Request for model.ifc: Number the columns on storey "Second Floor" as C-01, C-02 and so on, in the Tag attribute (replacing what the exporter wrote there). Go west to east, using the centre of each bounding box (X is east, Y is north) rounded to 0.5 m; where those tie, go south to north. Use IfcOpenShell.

First a look at what the model holds.

```python
import ifcopenshell
import ifcopenshell.util.element
import ifcopenshell.util.placement

model = ifcopenshell.open("model.ifc")
print(model.schema)
storey = next(s for s in model.by_type("IfcBuildingStorey") if s.Name == "Second Floor")
columns = [e for e in ifcopenshell.util.element.get_decomposition(storey) if e.is_a("IfcColumn")]
for e in sorted(columns, key=lambda e: e.id()):
    origin = ifcopenshell.util.placement.get_local_placement(e.ObjectPlacement)[:3, 3]
    print(e.id(), e.Tag, e.Name, origin.round(2) + 0.0, sep=" | ")
```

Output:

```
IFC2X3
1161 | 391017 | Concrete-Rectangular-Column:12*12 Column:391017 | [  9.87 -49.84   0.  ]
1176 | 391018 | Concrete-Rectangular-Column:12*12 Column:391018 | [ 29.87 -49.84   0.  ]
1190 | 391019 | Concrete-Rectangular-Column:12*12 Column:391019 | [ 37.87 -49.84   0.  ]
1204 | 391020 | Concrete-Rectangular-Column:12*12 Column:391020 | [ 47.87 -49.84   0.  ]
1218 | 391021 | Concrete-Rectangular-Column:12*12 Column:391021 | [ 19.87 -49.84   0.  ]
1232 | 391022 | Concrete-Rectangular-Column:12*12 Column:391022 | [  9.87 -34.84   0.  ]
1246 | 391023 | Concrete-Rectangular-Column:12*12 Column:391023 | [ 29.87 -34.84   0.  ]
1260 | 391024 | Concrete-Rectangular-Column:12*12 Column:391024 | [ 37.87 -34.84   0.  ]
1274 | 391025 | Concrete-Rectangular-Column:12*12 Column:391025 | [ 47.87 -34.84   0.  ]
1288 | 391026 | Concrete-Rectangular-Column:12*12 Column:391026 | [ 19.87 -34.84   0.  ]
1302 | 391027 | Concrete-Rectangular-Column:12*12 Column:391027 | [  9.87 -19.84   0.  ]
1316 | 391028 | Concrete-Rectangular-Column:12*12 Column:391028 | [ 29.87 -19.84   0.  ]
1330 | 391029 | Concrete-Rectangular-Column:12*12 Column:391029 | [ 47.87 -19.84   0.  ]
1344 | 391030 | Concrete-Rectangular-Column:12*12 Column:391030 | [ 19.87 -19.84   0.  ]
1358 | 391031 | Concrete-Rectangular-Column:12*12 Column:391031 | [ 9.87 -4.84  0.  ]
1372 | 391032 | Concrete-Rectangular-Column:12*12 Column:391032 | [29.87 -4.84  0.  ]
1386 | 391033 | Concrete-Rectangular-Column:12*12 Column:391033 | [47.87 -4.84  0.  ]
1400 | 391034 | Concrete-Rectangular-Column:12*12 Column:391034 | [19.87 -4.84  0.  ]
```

```python
import ifcopenshell
import ifcopenshell.geom
import ifcopenshell.util.element
import ifcopenshell.util.shape

model = ifcopenshell.open("model.ifc")
settings = ifcopenshell.geom.settings()
settings.set("use-world-coords", True)


def centre(element):
    shape = ifcopenshell.geom.create_shape(settings, element)
    return ifcopenshell.util.shape.get_bbox_centroid(shape.geometry)


storey = next(s for s in model.by_type("IfcBuildingStorey") if s.Name == "Second Floor")
columns = [e for e in ifcopenshell.util.element.get_decomposition(storey) if e.is_a("IfcColumn")]

# Insertion points can sit at a corner or the storey origin, so sort by the geometry (in metres).
centres = {e: centre(e) for e in columns}
columns.sort(key=lambda e: (round(centres[e][0] / 0.5), centres[e][1]))

for i, e in enumerate(columns, start=1):
    number = f"C-{i:02d}"
    e.Tag = number
    print(e.id(), number)

model.write("model_edited.ifc")
```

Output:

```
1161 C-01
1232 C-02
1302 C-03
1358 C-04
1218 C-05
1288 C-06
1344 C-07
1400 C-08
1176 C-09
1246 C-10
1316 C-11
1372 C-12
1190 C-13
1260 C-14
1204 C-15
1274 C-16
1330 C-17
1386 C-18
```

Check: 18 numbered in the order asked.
